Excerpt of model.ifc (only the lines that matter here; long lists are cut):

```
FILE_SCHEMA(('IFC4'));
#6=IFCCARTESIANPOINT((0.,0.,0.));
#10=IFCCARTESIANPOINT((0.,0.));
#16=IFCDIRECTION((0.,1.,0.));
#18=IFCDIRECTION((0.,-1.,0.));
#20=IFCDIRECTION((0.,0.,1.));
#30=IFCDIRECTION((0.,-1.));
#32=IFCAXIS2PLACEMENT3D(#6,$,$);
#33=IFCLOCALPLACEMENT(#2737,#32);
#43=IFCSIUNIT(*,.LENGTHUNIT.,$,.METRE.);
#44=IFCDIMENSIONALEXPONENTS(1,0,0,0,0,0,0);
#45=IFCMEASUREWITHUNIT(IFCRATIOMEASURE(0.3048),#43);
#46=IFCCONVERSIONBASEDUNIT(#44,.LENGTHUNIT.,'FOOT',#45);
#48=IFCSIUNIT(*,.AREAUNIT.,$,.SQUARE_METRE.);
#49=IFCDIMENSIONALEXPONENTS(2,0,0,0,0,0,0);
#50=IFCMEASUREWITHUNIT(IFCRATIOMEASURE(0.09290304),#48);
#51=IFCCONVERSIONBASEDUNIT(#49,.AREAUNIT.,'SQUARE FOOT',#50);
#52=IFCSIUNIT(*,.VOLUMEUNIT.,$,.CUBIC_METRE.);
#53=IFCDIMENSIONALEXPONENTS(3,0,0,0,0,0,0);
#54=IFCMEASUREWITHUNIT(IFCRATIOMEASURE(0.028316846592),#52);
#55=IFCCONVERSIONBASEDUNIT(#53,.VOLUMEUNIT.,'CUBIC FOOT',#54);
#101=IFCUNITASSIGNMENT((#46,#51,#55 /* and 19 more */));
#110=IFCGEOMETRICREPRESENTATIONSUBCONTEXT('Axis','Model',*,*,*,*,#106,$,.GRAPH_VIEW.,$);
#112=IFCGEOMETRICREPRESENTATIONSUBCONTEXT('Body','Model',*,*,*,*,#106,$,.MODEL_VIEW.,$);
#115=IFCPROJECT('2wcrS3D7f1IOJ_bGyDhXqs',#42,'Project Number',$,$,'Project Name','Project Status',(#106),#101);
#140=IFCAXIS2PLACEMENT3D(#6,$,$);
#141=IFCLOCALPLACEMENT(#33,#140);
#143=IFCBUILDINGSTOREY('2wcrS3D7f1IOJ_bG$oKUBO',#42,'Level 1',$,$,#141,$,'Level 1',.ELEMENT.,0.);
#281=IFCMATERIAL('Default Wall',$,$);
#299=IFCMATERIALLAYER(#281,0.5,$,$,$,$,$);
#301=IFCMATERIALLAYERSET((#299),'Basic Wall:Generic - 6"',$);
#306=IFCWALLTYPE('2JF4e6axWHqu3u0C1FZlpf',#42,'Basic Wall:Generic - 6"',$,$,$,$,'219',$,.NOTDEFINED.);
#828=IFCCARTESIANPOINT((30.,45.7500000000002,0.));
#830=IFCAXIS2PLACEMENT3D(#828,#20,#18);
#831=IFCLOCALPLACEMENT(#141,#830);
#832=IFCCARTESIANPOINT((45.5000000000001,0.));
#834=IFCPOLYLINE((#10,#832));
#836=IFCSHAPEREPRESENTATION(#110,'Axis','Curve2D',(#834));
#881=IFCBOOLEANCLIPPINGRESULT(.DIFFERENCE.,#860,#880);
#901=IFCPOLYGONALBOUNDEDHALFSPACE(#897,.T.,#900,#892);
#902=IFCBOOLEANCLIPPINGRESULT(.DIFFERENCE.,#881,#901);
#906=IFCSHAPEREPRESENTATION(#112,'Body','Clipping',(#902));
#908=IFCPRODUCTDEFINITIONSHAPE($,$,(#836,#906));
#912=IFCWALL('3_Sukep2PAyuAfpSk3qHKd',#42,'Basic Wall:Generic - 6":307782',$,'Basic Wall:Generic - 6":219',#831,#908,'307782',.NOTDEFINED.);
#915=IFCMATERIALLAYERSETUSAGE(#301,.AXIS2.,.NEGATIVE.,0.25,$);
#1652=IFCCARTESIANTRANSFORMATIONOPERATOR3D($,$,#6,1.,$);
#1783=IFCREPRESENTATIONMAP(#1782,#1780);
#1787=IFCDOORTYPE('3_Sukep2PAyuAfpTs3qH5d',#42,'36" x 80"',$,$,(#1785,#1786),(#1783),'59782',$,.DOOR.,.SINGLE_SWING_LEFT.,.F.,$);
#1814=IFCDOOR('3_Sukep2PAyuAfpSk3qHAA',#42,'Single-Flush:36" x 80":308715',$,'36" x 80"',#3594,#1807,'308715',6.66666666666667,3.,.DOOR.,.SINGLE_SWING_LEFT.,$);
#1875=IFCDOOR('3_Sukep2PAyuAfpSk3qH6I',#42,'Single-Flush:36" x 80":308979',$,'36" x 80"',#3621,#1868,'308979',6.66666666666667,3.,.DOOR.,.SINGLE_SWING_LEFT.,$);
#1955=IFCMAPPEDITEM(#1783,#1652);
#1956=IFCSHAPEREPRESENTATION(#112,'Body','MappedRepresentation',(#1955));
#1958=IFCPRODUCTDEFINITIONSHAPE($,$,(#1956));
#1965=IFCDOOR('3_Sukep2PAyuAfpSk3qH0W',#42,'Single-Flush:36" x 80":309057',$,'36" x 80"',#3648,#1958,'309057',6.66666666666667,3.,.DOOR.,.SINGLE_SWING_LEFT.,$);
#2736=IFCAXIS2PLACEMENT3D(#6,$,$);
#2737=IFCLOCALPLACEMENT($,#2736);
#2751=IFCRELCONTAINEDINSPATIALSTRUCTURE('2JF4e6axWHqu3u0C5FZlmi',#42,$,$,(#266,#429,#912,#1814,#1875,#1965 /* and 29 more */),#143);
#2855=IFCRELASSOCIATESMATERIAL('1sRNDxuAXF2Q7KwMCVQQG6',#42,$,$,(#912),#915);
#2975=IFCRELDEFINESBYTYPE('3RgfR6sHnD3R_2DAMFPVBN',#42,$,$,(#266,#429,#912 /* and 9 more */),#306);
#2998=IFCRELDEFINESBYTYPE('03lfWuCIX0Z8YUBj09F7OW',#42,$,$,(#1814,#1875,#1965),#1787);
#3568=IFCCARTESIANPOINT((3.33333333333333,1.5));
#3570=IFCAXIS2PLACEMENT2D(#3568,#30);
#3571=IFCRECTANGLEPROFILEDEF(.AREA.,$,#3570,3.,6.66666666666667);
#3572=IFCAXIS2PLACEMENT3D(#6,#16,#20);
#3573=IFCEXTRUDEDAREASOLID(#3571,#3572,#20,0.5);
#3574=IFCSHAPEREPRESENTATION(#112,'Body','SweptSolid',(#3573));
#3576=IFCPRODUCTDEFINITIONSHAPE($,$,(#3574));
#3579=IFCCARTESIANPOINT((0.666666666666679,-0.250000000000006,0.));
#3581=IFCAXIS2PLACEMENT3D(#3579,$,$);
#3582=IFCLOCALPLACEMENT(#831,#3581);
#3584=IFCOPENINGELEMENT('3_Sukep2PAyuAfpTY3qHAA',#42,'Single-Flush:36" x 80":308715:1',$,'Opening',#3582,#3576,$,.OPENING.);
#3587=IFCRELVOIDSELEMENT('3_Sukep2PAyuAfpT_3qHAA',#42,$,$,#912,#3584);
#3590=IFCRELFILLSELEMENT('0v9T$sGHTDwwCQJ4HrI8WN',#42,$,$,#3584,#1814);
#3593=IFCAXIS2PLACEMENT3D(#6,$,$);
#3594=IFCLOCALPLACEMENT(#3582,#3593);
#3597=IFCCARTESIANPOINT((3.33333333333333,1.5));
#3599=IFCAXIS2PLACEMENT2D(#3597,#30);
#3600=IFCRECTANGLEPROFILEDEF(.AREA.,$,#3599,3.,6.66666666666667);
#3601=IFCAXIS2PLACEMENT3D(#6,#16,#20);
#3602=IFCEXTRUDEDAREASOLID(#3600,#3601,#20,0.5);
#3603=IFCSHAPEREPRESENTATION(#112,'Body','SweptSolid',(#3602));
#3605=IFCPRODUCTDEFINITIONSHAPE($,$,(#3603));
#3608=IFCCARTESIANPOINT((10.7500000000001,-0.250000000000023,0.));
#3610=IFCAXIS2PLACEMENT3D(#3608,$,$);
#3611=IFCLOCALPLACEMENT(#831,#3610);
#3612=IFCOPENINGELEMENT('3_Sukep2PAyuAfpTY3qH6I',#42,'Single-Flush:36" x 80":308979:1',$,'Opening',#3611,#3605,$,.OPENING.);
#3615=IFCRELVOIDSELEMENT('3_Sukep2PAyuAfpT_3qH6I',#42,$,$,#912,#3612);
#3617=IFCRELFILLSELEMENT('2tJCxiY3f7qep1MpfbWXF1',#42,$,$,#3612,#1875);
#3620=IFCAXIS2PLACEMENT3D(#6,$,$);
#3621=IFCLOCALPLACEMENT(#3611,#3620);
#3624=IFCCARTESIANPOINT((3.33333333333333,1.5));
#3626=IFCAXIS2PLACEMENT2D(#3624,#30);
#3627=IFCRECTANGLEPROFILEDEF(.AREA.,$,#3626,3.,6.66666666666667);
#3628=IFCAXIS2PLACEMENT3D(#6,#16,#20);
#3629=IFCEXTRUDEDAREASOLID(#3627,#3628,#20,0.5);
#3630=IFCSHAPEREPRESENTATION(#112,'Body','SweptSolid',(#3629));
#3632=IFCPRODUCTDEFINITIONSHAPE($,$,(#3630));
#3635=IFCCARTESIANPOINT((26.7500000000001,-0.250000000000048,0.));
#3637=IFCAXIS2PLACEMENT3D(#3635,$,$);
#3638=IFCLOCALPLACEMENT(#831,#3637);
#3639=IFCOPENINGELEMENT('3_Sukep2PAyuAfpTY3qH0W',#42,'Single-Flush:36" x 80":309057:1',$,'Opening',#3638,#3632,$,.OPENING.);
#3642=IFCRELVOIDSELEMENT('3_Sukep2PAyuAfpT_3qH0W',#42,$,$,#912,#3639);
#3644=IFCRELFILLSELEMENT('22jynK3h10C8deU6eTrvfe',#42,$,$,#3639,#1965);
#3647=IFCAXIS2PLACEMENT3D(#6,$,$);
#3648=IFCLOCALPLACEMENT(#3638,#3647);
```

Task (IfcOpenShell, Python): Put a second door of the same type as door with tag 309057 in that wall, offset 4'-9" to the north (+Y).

```python
import ifcopenshell
import ifcopenshell.api.feature
import ifcopenshell.api.geometry
import ifcopenshell.api.root
import ifcopenshell.geom
import ifcopenshell.util.element
import ifcopenshell.util.placement
import ifcopenshell.util.shape
import ifcopenshell.util.unit

model = ifcopenshell.open("model.ifc")
unit_scale = ifcopenshell.util.unit.calculate_unit_scale(model)
settings = ifcopenshell.geom.settings()


def volume(element):
    """Net volume in cubic metres, openings subtracted."""
    shape = ifcopenshell.geom.create_shape(settings, element)
    return ifcopenshell.util.shape.get_volume(shape.geometry)


def reuse_history(source, copy):
    """copy_class also copies each property set's owner history, people and application; keep the originals."""
    for rel in copy.IsDefinedBy:
        if rel.is_a("IfcRelDefinesByProperties") and (history := rel.RelatingPropertyDefinition.OwnerHistory):
            rel.RelatingPropertyDefinition.OwnerHistory = source.OwnerHistory
            ifcopenshell.util.element.remove_deep2(model, history)


door = model.by_guid("3_Sukep2PAyuAfpSk3qH0W")
opening = door.FillsVoids[0].RelatingOpeningElement
wall = opening.VoidsElements[0].RelatingBuildingElement
before = volume(wall)
shift = ifcopenshell.util.placement.get_local_placement(wall.ObjectPlacement)[:3, 0] * -57 * 0.0254 / unit_scale

# copy_class copies the void relationship, type, container and properties, but no geometry.
new_opening = ifcopenshell.api.root.copy_class(model, product=opening)
new_opening.Representation = ifcopenshell.util.element.copy_deep(
    model, opening.Representation, exclude=["IfcGeometricRepresentationContext", "IfcRepresentationMap"]
)
new_opening.Name = 'Single-Flush:36" x 80"'
new_door = ifcopenshell.api.root.copy_class(model, product=door)
new_door.Representation = ifcopenshell.util.element.copy_deep(
    model, door.Representation, exclude=["IfcGeometricRepresentationContext", "IfcRepresentationMap"]
)
new_door.Name = 'Single-Flush:36" x 80"'
new_door.Tag = None
reuse_history(door, new_door)
ifcopenshell.api.feature.add_filling(model, opening=new_opening, element=new_door)

for old, new in ((opening, new_opening), (door, new_door)):
    matrix = ifcopenshell.util.placement.get_local_placement(old.ObjectPlacement)
    matrix[:3, 3] += shift
    ifcopenshell.api.geometry.edit_object_placement(model, product=new, matrix=matrix, is_si=False)

after = volume(wall)

print(f"wall volume {before:.3f} -> {after:.3f} m3")

model.write("model_rev.ifc")
```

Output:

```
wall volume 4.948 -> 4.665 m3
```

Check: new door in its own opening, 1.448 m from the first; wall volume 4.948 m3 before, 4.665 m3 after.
